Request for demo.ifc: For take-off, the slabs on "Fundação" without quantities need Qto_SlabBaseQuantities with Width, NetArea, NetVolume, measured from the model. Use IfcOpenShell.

First a look at what the model holds.

```python
import ifcopenshell
import ifcopenshell.util.element
import ifcopenshell.util.unit

model = ifcopenshell.open("demo.ifc")
print(model.schema)
for unit_type in ("LENGTHUNIT", "AREAUNIT", "VOLUMEUNIT"):
    print(unit_type, ifcopenshell.util.unit.calculate_unit_scale(model, unit_type))
storey = next(s for s in model.by_type("IfcBuildingStorey") if s.Name == "Fundação")
slabs = [e for e in ifcopenshell.util.element.get_decomposition(storey) if e.is_a("IfcSlab")]
for e in sorted(slabs, key=lambda e: e.id()):
    print(e.id(), e.is_a(), e.Name, list(ifcopenshell.util.element.get_psets(e, qtos_only=True)), sep=" | ")
```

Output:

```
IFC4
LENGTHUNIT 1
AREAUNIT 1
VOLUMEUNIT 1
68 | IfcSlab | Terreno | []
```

```python
import ifcopenshell
import ifcopenshell.api.pset
import ifcopenshell.geom
import ifcopenshell.util.element
import ifcopenshell.util.shape
import ifcopenshell.util.unit

model = ifcopenshell.open("demo.ifc")
unit_scale = ifcopenshell.util.unit.calculate_unit_scale(model)
area_scale = ifcopenshell.util.unit.calculate_unit_scale(model, "AREAUNIT")
volume_scale = ifcopenshell.util.unit.calculate_unit_scale(model, "VOLUMEUNIT")
settings = ifcopenshell.geom.settings()

storey = next(s for s in model.by_type("IfcBuildingStorey") if s.Name == "Fundação")
slabs = [e for e in ifcopenshell.util.element.get_decomposition(storey) if e.is_a("IfcSlab")]

for e in sorted(slabs, key=lambda e: e.id()):
    if ifcopenshell.util.element.get_psets(e, qtos_only=True, should_inherit=False):
        continue
    # Geometry comes back in metres, in the element's own axes.
    shape = ifcopenshell.geom.create_shape(settings, e)
    values = {
        "Width": ifcopenshell.util.shape.get_z(shape.geometry) / unit_scale,
        "NetArea": ifcopenshell.util.shape.get_footprint_area(shape.geometry) / area_scale,
        "NetVolume": ifcopenshell.util.shape.get_volume(shape.geometry) / volume_scale,
    }
    qto = ifcopenshell.api.pset.add_qto(model, product=e, name="Qto_SlabBaseQuantities")
    ifcopenshell.api.pset.edit_qto(model, qto=qto, properties=values)
    print(e.id(), {k: round(v, 3) for k, v in values.items()})

model.write("demo_edited.ifc")
```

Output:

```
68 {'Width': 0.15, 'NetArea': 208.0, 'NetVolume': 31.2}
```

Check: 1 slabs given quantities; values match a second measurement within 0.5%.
